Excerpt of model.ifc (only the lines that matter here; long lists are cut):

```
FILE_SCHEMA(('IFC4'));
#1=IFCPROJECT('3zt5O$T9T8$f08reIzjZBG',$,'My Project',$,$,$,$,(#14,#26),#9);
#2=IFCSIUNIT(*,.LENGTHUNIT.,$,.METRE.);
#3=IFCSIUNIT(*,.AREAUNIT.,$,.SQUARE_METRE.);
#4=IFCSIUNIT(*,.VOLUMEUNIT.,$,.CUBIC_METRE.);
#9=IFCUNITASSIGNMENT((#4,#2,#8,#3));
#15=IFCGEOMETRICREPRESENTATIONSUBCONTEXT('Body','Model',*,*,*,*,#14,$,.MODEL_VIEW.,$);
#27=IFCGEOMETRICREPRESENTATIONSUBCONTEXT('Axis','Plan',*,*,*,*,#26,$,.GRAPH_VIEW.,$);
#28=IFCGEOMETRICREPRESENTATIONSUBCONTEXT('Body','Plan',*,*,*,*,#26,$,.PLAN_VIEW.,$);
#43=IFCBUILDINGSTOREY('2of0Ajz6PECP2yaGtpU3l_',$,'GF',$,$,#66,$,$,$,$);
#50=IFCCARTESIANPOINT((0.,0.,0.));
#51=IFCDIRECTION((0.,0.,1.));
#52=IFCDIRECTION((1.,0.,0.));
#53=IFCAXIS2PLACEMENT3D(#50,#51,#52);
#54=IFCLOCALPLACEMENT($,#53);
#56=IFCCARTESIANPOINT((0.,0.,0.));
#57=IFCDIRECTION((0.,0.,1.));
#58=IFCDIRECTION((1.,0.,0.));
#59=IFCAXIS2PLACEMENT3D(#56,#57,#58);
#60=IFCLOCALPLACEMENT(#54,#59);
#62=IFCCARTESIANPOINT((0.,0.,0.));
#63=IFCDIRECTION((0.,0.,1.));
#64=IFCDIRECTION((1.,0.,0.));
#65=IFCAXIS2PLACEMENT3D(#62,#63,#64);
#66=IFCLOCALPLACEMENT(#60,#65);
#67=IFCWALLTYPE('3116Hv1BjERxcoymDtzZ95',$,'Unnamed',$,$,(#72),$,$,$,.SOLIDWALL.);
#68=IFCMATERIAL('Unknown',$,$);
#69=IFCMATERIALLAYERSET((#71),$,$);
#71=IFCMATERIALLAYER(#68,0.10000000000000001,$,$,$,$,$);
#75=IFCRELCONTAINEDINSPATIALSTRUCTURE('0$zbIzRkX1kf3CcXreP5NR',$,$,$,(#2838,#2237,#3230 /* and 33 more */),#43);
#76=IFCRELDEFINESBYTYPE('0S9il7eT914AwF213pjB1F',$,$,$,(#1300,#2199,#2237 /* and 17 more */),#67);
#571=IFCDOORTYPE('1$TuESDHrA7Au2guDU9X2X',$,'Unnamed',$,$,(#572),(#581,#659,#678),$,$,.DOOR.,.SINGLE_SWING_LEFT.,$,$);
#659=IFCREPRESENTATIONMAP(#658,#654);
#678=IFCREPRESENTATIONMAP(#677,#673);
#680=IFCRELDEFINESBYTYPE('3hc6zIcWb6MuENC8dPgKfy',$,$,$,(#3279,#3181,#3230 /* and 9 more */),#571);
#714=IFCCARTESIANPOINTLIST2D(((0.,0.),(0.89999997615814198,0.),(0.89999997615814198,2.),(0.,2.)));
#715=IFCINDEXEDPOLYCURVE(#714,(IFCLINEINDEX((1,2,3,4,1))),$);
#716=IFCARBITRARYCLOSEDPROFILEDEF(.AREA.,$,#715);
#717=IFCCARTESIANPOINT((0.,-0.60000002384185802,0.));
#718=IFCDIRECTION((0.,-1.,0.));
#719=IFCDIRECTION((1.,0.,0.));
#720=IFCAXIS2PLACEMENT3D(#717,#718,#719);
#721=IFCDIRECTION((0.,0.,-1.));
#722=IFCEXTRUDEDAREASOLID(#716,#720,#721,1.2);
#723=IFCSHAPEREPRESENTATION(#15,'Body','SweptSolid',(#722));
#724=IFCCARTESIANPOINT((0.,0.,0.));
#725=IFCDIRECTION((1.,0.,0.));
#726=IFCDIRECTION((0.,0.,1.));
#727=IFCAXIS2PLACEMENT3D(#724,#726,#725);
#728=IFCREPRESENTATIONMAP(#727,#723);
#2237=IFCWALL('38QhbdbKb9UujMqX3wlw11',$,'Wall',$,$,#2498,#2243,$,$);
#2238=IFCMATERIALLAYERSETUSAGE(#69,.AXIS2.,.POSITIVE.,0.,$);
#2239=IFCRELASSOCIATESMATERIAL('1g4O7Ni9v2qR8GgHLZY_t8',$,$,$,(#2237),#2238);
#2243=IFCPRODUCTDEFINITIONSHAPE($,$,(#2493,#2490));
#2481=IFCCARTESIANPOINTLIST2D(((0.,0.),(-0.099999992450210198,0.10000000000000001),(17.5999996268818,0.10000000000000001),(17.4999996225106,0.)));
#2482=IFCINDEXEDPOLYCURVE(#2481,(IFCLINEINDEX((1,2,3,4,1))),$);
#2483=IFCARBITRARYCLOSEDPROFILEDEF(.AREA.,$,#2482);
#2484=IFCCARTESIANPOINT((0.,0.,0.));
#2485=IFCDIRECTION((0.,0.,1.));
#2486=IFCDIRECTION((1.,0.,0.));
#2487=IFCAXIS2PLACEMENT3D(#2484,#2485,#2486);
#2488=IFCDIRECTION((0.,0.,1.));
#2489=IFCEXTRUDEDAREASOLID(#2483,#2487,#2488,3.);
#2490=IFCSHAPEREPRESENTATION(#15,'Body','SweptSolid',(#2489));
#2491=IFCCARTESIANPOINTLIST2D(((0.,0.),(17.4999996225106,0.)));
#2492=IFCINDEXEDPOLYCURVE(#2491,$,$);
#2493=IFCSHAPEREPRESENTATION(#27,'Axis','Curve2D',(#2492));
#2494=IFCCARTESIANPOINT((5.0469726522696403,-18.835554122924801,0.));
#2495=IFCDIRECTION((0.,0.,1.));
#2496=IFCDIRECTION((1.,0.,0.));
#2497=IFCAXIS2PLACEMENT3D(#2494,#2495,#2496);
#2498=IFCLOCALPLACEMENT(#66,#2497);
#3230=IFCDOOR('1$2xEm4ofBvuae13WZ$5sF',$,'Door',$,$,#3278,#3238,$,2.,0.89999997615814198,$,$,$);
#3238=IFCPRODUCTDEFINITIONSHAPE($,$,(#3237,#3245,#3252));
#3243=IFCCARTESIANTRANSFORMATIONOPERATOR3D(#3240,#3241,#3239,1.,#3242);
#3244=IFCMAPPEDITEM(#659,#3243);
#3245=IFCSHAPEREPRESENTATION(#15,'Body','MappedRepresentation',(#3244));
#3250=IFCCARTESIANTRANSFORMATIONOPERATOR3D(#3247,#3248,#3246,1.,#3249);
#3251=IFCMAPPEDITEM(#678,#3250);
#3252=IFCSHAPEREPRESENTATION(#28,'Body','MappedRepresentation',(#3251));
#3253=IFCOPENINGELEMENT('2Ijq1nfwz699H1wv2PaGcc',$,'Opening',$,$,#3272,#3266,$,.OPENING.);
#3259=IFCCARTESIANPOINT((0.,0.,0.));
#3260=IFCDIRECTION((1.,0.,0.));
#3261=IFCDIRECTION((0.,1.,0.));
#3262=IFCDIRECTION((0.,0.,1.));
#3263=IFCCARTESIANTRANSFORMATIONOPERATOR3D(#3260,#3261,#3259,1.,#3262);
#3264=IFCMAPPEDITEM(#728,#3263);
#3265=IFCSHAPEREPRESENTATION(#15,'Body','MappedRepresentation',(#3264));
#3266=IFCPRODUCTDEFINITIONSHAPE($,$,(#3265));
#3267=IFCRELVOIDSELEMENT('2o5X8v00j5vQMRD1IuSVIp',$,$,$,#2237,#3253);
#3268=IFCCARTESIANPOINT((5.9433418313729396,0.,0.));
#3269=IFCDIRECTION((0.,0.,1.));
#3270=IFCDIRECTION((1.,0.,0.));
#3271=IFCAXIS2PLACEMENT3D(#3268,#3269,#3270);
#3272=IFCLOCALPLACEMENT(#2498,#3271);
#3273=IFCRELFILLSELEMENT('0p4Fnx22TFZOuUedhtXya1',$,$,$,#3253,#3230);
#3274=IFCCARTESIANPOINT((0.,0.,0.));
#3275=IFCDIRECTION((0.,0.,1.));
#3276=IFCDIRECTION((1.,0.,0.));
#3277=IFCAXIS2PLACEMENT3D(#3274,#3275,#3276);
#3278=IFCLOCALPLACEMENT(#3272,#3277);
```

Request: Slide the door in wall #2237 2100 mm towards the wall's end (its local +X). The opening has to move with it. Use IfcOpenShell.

```python
import ifcopenshell
import ifcopenshell.api.geometry
import ifcopenshell.util.placement
import ifcopenshell.util.unit

model = ifcopenshell.open("model.ifc")
unit_scale = ifcopenshell.util.unit.calculate_unit_scale(model)

door = model.by_guid("1$2xEm4ofBvuae13WZ$5sF")
opening = door.FillsVoids[0].RelatingOpeningElement
wall = opening.VoidsElements[0].RelatingBuildingElement

wall_matrix = ifcopenshell.util.placement.get_local_placement(wall.ObjectPlacement)
shift = wall_matrix[:3, 0] * 2.1 / unit_scale
before = ifcopenshell.util.placement.get_local_placement(door.ObjectPlacement)[:3, 3].copy()

# The door is placed relative to its opening, so it follows when the opening moves.
matrix = ifcopenshell.util.placement.get_local_placement(opening.ObjectPlacement)
matrix[:3, 3] += shift
ifcopenshell.api.geometry.edit_object_placement(
    model, product=opening, matrix=matrix, is_si=False, should_transform_children=True
)

after = ifcopenshell.util.placement.get_local_placement(door.ObjectPlacement)[:3, 3]
print("door moved by", (after - before).round(3) + 0.0)

model.write("model_rev.ifc")
```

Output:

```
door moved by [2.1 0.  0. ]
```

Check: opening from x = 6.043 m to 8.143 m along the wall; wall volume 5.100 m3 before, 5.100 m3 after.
